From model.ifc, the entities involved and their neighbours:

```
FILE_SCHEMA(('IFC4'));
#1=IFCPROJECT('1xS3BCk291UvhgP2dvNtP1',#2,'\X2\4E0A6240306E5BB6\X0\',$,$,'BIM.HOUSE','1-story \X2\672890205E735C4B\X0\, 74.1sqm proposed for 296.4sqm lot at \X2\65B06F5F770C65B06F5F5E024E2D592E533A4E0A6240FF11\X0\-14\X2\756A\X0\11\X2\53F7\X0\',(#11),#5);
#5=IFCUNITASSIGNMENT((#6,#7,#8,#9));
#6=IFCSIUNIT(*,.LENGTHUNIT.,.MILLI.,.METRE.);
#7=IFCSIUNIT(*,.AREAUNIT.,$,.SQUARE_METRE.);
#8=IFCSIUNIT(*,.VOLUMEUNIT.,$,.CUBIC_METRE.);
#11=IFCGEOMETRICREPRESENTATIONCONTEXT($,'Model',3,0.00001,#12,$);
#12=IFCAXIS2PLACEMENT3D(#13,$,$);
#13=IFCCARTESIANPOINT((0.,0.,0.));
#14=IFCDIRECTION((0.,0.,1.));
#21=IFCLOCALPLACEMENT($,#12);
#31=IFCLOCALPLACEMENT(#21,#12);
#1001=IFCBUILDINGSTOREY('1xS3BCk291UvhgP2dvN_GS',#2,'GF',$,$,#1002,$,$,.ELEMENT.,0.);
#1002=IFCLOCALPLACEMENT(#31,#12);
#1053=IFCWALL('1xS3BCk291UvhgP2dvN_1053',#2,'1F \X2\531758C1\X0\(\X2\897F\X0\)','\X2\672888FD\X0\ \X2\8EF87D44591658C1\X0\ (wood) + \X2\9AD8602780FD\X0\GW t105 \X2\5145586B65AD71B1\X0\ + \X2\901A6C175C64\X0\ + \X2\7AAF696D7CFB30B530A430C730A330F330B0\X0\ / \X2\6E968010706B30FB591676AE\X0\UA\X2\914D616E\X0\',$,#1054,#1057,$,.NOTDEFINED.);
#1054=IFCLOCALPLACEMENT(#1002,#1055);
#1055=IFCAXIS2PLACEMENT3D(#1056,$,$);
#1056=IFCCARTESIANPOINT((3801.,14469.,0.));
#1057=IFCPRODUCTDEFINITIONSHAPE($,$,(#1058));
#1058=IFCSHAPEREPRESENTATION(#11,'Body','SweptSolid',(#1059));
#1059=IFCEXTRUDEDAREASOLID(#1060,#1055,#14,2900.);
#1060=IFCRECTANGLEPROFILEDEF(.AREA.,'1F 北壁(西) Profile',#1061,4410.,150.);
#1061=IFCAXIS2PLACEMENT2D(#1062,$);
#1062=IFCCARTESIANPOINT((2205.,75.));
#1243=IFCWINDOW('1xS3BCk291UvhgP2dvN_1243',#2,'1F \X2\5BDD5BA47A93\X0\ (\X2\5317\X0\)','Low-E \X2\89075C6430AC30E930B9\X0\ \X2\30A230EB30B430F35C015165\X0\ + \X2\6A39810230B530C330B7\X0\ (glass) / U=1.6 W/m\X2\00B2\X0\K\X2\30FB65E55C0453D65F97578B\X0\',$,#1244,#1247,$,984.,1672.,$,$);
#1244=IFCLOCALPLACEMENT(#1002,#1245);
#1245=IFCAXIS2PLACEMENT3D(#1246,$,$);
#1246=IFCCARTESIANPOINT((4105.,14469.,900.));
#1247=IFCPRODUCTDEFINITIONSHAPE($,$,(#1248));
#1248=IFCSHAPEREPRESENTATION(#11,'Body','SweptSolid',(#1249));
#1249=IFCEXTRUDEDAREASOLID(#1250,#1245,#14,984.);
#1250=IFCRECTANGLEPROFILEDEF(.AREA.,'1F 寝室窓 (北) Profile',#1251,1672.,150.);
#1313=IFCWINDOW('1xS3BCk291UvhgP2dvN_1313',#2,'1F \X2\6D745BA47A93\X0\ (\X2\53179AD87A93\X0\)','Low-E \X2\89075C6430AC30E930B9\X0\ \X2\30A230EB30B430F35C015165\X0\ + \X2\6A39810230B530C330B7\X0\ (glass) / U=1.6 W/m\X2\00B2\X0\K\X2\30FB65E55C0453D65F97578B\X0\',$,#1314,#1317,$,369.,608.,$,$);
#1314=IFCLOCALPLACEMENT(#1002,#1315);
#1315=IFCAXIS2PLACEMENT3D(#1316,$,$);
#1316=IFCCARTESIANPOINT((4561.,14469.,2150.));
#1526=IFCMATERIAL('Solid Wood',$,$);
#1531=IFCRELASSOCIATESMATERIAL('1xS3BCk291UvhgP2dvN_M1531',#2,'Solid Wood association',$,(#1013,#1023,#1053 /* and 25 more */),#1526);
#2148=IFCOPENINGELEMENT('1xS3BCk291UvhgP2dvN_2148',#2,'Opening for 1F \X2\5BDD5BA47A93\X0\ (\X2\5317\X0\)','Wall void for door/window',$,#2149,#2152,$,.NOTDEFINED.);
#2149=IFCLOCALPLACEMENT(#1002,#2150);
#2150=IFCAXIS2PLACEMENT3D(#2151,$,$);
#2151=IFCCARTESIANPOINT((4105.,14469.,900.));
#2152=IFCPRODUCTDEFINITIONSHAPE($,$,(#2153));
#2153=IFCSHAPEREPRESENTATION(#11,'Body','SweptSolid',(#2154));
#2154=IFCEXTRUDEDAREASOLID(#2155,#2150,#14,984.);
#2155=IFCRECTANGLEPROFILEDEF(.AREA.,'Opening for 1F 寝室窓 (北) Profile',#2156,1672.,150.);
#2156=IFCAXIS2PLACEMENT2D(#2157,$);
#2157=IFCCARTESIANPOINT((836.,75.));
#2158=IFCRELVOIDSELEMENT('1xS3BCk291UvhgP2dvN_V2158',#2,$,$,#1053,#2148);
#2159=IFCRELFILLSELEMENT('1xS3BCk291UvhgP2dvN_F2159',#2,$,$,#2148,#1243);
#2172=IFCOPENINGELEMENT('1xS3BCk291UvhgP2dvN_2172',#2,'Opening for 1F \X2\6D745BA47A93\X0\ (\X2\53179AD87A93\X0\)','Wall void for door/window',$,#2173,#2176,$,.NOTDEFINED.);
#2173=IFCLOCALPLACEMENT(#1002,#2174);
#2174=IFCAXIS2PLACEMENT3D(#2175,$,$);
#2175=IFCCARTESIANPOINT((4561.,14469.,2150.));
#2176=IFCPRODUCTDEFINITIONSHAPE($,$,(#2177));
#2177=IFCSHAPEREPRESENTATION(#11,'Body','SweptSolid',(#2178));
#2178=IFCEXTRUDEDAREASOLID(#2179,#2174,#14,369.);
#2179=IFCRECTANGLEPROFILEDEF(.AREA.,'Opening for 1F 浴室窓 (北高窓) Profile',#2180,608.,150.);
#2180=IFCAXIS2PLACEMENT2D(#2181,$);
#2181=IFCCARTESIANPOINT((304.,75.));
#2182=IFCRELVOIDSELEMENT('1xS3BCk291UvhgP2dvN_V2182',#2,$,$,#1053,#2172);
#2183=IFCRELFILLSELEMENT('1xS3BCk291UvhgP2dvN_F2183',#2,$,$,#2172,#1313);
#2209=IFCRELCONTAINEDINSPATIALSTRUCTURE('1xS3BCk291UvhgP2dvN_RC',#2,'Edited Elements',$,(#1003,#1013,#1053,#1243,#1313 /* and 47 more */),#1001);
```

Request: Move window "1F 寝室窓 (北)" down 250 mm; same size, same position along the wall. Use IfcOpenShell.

```python
import numpy as np
import ifcopenshell
import ifcopenshell.api.geometry
import ifcopenshell.util.placement
import ifcopenshell.util.unit

model = ifcopenshell.open("model.ifc")
unit_scale = ifcopenshell.util.unit.calculate_unit_scale(model)

window = model.by_id(1243)
opening = window.FillsVoids[0].RelatingOpeningElement
dz = -250.0

shift = np.array([0.0, 0.0, dz])
# The window is not placed relative to its opening, so move both.
for product in (opening, window):
    matrix = ifcopenshell.util.placement.get_local_placement(product.ObjectPlacement)
    matrix[:3, 3] += shift
    ifcopenshell.api.geometry.edit_object_placement(model, product=product, matrix=matrix, is_si=False)

print(f"moved by {dz * unit_scale:+.3f} m")

model.write("model_v2.ifc")
```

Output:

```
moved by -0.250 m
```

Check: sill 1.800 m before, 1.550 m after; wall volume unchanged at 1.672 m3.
